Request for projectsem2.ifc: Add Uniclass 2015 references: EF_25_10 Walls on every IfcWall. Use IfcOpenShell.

First a look at what the model holds.

```python
import ifcopenshell

model = ifcopenshell.open("projectsem2.ifc")
print(model.schema)
print("classifications:", [c.Name for c in model.by_type("IfcClassification")])
for ifc_class in ("IfcDoor", "IfcRoof", "IfcStair", "IfcWall", "IfcWindow"):
    print(ifc_class, len(model.by_type(ifc_class)))
```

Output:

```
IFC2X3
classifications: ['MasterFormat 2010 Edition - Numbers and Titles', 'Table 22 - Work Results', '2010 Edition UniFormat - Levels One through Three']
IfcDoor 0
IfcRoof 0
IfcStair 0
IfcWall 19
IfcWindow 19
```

```python
import ifcopenshell
import ifcopenshell.api.classification

model = ifcopenshell.open("projectsem2.ifc")

# IFC2X3 requires Source and Edition and has no link from the project to the system.
system = model.create_entity("IfcClassification", Source="NBS", Edition="2015", Name="Uniclass 2015")

codes = {
    "IfcWall": ("EF_25_10", "Walls"),
}
for ifc_class, (code, name) in codes.items():
    products = model.by_type(ifc_class)
    ifcopenshell.api.classification.add_reference(
        model, products=products, classification=system, identification=code, name=name
    )
    print(code, len(products))

model.write("projectsem2_rev.ifc")
```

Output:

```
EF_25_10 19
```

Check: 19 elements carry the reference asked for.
